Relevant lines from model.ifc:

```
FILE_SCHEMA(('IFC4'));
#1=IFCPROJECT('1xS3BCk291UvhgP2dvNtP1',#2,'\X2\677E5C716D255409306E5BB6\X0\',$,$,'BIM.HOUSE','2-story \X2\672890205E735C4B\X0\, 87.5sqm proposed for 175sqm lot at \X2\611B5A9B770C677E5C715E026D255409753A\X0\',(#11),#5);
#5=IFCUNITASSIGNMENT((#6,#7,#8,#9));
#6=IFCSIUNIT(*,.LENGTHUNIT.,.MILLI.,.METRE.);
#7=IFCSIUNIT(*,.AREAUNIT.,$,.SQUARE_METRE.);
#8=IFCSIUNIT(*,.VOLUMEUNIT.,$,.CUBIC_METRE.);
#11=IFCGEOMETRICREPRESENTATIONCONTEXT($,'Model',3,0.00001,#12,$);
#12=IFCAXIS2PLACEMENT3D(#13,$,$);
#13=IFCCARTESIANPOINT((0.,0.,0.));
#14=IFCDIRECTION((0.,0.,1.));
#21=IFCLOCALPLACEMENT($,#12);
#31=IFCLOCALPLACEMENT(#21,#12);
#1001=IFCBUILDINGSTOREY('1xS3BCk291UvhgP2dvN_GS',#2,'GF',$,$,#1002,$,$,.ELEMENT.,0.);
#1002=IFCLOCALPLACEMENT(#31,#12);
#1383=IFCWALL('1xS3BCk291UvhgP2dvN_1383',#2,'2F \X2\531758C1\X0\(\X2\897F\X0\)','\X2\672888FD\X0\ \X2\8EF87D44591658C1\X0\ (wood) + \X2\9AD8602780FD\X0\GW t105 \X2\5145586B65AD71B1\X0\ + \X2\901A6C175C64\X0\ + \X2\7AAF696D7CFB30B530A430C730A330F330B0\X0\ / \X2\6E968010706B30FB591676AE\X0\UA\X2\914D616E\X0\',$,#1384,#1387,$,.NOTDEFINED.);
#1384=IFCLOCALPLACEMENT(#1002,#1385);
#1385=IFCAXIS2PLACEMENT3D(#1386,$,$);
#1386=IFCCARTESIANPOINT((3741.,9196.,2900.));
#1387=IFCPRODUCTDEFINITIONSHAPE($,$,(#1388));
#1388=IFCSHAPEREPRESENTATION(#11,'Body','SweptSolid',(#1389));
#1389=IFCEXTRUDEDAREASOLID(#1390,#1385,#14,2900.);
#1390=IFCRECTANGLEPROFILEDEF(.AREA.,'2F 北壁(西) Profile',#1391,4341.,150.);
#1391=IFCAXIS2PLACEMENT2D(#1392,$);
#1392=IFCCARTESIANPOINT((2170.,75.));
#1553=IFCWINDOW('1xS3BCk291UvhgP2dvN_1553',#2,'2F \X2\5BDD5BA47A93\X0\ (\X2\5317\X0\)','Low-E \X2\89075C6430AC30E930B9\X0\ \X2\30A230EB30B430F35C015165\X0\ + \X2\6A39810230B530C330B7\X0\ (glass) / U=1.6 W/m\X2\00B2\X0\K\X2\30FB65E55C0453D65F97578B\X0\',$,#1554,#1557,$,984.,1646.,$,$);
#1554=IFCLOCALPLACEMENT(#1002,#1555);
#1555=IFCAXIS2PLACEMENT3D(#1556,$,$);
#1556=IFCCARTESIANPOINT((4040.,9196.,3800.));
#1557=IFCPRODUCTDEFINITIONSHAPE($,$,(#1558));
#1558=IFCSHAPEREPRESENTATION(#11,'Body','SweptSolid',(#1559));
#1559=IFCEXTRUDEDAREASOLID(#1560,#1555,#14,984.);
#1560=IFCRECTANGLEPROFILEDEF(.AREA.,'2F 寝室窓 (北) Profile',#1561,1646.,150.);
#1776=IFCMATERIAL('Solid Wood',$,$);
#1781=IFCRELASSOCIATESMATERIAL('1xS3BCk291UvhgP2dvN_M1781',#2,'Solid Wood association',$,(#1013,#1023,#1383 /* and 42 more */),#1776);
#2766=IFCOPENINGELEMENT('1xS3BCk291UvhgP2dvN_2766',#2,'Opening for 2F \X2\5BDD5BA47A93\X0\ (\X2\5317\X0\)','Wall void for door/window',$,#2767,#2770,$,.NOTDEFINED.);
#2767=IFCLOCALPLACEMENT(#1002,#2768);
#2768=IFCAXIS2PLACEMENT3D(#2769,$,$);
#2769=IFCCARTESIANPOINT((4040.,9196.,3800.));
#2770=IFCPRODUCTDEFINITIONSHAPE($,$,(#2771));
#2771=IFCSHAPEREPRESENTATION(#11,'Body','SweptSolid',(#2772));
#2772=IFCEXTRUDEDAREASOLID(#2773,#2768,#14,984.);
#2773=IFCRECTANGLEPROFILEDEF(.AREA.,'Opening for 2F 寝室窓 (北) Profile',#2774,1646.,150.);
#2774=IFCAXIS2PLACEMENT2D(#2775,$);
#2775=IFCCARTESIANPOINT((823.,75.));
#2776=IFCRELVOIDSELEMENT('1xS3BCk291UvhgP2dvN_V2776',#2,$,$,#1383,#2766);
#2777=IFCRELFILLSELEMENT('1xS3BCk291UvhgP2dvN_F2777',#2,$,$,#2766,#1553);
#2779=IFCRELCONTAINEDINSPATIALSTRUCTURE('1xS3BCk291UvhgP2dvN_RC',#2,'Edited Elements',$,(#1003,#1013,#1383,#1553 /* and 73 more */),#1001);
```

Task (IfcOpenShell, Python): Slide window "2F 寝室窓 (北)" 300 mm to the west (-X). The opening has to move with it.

```python
import ifcopenshell
import ifcopenshell.api.geometry
import ifcopenshell.util.placement
import ifcopenshell.util.unit

model = ifcopenshell.open("model.ifc")
unit_scale = ifcopenshell.util.unit.calculate_unit_scale(model)

window = model.by_guid("1xS3BCk291UvhgP2dvN_1553")
opening = window.FillsVoids[0].RelatingOpeningElement
wall = opening.VoidsElements[0].RelatingBuildingElement

wall_matrix = ifcopenshell.util.placement.get_local_placement(wall.ObjectPlacement)
shift = wall_matrix[:3, 0] * -0.3 / unit_scale
before = ifcopenshell.util.placement.get_local_placement(window.ObjectPlacement)[:3, 3].copy()

# The window is not placed relative to its opening, so move both.
for product in (opening, window):
    matrix = ifcopenshell.util.placement.get_local_placement(product.ObjectPlacement)
    matrix[:3, 3] += shift
    ifcopenshell.api.geometry.edit_object_placement(model, product=product, matrix=matrix, is_si=False)

after = ifcopenshell.util.placement.get_local_placement(window.ObjectPlacement)[:3, 3]
print("window moved by", (after - before).round(3) + 0.0)

model.write("model_updated.ifc")
```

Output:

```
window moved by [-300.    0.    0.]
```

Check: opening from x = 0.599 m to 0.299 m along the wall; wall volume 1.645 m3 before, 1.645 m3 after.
